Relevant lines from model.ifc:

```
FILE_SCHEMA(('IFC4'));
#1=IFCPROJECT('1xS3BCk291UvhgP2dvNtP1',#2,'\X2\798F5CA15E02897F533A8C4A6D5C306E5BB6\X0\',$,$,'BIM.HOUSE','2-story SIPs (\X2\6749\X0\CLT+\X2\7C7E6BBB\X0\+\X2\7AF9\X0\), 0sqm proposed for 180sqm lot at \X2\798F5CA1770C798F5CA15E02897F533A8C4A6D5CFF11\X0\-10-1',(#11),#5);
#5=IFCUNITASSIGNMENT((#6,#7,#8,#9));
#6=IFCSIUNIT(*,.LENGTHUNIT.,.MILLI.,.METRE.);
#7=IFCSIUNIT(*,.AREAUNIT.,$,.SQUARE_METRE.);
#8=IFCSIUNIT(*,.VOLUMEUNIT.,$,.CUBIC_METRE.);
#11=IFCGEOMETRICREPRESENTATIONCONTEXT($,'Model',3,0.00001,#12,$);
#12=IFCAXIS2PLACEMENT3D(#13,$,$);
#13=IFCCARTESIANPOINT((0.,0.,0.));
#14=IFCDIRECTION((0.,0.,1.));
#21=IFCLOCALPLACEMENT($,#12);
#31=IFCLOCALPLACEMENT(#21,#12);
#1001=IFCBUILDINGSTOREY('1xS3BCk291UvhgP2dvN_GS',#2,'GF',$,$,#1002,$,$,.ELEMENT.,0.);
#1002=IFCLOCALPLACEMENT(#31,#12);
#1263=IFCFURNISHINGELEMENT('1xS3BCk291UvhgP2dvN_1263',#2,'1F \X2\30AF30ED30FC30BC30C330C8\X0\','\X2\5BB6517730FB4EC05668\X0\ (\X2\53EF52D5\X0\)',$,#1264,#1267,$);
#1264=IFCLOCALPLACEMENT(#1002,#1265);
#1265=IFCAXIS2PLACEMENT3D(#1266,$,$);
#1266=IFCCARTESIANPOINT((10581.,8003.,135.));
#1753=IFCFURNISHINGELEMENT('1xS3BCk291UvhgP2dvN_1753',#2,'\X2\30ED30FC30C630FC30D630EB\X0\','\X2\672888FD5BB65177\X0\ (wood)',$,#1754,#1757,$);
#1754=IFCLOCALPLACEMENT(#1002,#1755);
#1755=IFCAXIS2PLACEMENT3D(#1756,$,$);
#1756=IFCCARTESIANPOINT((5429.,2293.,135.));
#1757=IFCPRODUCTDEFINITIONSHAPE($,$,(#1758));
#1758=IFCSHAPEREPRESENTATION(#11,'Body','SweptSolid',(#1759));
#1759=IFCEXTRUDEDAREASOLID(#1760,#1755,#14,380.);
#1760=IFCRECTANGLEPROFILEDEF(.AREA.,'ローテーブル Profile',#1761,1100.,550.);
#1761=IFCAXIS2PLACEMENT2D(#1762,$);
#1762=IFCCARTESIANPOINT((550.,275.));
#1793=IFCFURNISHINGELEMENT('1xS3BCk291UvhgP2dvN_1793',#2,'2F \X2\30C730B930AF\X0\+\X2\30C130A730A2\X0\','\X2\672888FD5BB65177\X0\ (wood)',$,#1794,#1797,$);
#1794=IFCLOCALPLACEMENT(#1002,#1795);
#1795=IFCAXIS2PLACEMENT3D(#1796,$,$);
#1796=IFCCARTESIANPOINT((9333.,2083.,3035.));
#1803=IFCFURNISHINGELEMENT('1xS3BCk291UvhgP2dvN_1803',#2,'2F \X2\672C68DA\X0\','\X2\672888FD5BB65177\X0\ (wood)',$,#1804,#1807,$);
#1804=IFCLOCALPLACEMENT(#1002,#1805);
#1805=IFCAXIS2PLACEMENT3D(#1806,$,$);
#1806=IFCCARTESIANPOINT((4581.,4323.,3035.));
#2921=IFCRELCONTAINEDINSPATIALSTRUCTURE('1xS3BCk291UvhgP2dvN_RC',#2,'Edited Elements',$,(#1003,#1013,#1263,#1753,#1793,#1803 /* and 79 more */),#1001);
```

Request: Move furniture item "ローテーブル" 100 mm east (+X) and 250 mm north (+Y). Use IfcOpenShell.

```python
import ifcopenshell
import ifcopenshell.api.geometry
import ifcopenshell.util.placement
import ifcopenshell.util.unit

model = ifcopenshell.open("model.ifc")
unit_scale = ifcopenshell.util.unit.calculate_unit_scale(model)

item = model.by_guid("1xS3BCk291UvhgP2dvN_1753")
matrix = ifcopenshell.util.placement.get_local_placement(item.ObjectPlacement)
matrix[0, 3] += 0.1 / unit_scale
matrix[1, 3] += 0.25 / unit_scale
ifcopenshell.api.geometry.edit_object_placement(model, product=item, matrix=matrix, is_si=False)

print(ifcopenshell.util.placement.get_local_placement(item.ObjectPlacement).round(3) + 0.0)

model.write("model-out.ifc")
```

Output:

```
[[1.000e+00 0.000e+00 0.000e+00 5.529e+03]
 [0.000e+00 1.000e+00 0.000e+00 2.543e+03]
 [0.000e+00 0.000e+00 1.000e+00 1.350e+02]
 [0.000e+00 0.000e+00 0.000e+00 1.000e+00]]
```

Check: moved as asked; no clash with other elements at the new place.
